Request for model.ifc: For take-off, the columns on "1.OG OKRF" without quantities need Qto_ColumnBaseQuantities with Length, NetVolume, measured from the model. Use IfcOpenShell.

First a look at what the model holds.

```python
import ifcopenshell
import ifcopenshell.util.element
import ifcopenshell.util.unit

model = ifcopenshell.open("model.ifc")
print(model.schema)
for unit_type in ("LENGTHUNIT", "AREAUNIT", "VOLUMEUNIT"):
    print(unit_type, ifcopenshell.util.unit.calculate_unit_scale(model, unit_type))
storey = next(s for s in model.by_type("IfcBuildingStorey") if s.Name == "1.OG OKRF")
columns = [e for e in ifcopenshell.util.element.get_decomposition(storey) if e.is_a("IfcColumn")]
for e in sorted(columns, key=lambda e: e.id()):
    print(e.id(), e.is_a(), e.Name, list(ifcopenshell.util.element.get_psets(e, qtos_only=True)), sep=" | ")
```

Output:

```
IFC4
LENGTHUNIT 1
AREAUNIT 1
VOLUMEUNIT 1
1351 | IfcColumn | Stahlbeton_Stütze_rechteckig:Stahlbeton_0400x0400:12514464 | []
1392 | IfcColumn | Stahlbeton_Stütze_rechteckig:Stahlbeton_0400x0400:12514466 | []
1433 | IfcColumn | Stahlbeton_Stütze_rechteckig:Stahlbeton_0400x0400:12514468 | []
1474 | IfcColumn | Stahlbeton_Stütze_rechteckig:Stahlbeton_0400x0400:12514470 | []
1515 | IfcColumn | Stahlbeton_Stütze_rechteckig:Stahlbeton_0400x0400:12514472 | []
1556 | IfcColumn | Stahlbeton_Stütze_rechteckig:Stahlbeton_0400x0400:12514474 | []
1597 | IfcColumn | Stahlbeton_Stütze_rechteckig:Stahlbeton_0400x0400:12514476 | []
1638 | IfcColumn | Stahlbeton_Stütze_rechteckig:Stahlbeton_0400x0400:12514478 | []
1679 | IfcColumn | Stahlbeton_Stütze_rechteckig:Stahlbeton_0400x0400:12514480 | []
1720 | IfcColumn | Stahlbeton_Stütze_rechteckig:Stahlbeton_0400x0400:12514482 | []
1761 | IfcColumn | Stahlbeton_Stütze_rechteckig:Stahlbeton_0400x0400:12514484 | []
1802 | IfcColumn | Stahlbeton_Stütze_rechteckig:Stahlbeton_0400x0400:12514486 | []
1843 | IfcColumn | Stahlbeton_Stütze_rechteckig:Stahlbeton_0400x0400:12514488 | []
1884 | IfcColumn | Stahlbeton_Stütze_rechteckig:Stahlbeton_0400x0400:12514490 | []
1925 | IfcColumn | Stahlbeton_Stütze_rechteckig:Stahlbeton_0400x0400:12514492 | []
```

```python
import ifcopenshell
import ifcopenshell.api.pset
import ifcopenshell.geom
import ifcopenshell.util.element
import ifcopenshell.util.shape
import ifcopenshell.util.unit

model = ifcopenshell.open("model.ifc")
unit_scale = ifcopenshell.util.unit.calculate_unit_scale(model)
volume_scale = ifcopenshell.util.unit.calculate_unit_scale(model, "VOLUMEUNIT")
settings = ifcopenshell.geom.settings()

storey = next(s for s in model.by_type("IfcBuildingStorey") if s.Name == "1.OG OKRF")
columns = [e for e in ifcopenshell.util.element.get_decomposition(storey) if e.is_a("IfcColumn")]

for e in sorted(columns, key=lambda e: e.id()):
    if ifcopenshell.util.element.get_psets(e, qtos_only=True, should_inherit=False):
        continue
    # Geometry comes back in metres, in the element's own axes.
    shape = ifcopenshell.geom.create_shape(settings, e)
    values = {
        "Length": ifcopenshell.util.shape.get_z(shape.geometry) / unit_scale,
        "NetVolume": ifcopenshell.util.shape.get_volume(shape.geometry) / volume_scale,
    }
    qto = ifcopenshell.api.pset.add_qto(model, product=e, name="Qto_ColumnBaseQuantities")
    ifcopenshell.api.pset.edit_qto(model, qto=qto, properties=values)
    print(e.id(), {k: round(v, 3) for k, v in values.items()})

model.write("model-out.ifc")
```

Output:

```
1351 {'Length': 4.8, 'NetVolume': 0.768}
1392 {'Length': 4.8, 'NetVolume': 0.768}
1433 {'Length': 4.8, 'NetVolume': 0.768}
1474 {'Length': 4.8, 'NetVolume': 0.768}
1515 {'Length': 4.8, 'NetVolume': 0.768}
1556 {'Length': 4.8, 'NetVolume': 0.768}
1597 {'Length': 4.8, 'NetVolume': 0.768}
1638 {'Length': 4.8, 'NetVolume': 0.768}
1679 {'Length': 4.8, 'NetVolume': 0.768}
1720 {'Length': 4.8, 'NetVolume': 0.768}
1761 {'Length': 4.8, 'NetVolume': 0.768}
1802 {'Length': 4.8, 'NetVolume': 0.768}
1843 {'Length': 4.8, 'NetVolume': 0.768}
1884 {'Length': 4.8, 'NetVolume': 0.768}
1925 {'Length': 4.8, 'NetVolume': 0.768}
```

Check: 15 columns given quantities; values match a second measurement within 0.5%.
